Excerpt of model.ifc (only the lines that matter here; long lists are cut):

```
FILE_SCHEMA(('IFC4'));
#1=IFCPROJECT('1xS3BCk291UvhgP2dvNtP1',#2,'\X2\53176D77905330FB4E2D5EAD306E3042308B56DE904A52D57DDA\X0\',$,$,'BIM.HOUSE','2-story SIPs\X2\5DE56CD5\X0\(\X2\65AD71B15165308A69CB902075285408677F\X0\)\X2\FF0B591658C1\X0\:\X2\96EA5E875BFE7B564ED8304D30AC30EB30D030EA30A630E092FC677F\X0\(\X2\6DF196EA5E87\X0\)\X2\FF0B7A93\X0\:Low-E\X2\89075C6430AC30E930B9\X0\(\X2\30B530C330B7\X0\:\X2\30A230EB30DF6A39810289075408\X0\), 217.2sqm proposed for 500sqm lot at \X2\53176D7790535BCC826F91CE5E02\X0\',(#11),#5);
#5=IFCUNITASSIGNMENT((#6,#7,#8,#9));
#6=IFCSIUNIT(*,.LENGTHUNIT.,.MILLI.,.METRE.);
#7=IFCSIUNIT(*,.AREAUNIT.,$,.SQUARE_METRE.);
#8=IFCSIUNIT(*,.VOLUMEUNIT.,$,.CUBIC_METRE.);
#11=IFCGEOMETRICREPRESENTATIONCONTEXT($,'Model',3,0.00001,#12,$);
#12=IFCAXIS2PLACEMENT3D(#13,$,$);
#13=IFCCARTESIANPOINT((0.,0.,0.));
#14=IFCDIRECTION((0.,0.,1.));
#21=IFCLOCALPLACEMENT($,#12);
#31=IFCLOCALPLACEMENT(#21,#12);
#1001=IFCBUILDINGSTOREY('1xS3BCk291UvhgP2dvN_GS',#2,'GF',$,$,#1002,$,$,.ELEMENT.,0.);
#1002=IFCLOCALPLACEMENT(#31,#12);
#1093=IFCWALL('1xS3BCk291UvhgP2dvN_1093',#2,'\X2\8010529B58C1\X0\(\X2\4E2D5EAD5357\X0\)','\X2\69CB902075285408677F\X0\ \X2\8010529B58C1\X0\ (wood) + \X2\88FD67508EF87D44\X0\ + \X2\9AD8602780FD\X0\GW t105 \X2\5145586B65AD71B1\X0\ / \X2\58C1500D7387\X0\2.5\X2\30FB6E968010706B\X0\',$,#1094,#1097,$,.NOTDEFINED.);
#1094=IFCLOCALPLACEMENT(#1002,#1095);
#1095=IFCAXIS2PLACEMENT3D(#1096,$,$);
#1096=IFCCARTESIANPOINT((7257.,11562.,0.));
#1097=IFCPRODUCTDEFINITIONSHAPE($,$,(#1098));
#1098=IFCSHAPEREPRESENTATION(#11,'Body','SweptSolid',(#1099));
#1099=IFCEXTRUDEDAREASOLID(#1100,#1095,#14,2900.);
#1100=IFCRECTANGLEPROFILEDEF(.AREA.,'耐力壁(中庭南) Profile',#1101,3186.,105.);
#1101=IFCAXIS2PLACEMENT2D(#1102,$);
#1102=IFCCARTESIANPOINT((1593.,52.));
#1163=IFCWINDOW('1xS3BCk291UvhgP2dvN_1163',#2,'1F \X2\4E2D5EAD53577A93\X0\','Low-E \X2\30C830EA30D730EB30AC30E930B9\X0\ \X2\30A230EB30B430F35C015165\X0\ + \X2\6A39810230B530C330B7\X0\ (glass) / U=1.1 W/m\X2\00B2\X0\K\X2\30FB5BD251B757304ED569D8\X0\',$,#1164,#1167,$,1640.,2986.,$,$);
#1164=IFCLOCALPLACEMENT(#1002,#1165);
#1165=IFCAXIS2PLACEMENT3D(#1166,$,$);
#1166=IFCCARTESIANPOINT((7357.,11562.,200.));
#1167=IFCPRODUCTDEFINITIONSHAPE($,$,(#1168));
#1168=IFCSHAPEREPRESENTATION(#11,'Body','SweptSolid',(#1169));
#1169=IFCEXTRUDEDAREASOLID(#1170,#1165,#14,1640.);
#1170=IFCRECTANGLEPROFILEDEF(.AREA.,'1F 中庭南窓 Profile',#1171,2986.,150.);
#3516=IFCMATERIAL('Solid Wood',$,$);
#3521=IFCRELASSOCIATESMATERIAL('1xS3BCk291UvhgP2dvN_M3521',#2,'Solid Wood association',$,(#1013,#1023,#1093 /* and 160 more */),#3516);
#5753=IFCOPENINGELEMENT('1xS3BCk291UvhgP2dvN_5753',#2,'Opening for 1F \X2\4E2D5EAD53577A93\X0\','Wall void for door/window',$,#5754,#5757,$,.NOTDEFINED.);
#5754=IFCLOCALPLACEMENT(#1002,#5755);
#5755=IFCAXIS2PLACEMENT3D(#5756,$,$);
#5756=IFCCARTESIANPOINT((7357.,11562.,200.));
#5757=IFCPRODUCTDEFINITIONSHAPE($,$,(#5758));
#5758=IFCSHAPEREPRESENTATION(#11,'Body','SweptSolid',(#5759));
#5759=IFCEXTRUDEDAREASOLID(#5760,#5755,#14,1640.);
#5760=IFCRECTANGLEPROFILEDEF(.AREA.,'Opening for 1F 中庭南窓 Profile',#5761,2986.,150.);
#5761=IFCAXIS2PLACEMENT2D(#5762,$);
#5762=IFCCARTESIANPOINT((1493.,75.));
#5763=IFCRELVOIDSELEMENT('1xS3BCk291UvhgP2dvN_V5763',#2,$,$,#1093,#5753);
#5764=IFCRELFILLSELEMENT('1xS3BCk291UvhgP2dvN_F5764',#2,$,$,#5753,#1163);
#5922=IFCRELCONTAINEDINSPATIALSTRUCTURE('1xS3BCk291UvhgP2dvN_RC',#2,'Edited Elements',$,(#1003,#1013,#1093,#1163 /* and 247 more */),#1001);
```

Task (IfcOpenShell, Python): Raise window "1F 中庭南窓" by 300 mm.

```python
import numpy as np
import ifcopenshell
import ifcopenshell.api.geometry
import ifcopenshell.util.placement
import ifcopenshell.util.unit

model = ifcopenshell.open("model.ifc")
unit_scale = ifcopenshell.util.unit.calculate_unit_scale(model)

window = model.by_guid("1xS3BCk291UvhgP2dvN_1163")
opening = window.FillsVoids[0].RelatingOpeningElement
dz = 300.0

shift = np.array([0.0, 0.0, dz])
# The window is not placed relative to its opening, so move both.
for product in (opening, window):
    matrix = ifcopenshell.util.placement.get_local_placement(product.ObjectPlacement)
    matrix[:3, 3] += shift
    ifcopenshell.api.geometry.edit_object_placement(model, product=product, matrix=matrix, is_si=False)

print(f"moved by {dz * unit_scale:+.3f} m")

model.write("model-out.ifc")
```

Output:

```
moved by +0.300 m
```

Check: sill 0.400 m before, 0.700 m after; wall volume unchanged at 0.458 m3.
